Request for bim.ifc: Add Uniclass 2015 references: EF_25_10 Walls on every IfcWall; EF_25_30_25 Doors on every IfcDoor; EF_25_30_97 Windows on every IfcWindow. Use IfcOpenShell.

First a look at what the model holds.

```python
import ifcopenshell

model = ifcopenshell.open("bim.ifc")
print(model.schema)
print("classifications:", [c.Name for c in model.by_type("IfcClassification")])
for ifc_class in ("IfcDoor", "IfcRoof", "IfcStair", "IfcWall", "IfcWindow"):
    print(ifc_class, len(model.by_type(ifc_class)))
```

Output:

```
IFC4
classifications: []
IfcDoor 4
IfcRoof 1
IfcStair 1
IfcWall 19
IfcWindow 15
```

```python
import ifcopenshell
import ifcopenshell.api.classification

model = ifcopenshell.open("bim.ifc")

system = ifcopenshell.api.classification.add_classification(model, classification="Uniclass 2015")

codes = {
    "IfcWall": ("EF_25_10", "Walls"),
    "IfcDoor": ("EF_25_30_25", "Doors"),
    "IfcWindow": ("EF_25_30_97", "Windows"),
}
for ifc_class, (code, name) in codes.items():
    products = model.by_type(ifc_class)
    ifcopenshell.api.classification.add_reference(
        model, products=products, classification=system, identification=code, name=name
    )
    print(code, len(products))

model.write("bim_rev.ifc")
```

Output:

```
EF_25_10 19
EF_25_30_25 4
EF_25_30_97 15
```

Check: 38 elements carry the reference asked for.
